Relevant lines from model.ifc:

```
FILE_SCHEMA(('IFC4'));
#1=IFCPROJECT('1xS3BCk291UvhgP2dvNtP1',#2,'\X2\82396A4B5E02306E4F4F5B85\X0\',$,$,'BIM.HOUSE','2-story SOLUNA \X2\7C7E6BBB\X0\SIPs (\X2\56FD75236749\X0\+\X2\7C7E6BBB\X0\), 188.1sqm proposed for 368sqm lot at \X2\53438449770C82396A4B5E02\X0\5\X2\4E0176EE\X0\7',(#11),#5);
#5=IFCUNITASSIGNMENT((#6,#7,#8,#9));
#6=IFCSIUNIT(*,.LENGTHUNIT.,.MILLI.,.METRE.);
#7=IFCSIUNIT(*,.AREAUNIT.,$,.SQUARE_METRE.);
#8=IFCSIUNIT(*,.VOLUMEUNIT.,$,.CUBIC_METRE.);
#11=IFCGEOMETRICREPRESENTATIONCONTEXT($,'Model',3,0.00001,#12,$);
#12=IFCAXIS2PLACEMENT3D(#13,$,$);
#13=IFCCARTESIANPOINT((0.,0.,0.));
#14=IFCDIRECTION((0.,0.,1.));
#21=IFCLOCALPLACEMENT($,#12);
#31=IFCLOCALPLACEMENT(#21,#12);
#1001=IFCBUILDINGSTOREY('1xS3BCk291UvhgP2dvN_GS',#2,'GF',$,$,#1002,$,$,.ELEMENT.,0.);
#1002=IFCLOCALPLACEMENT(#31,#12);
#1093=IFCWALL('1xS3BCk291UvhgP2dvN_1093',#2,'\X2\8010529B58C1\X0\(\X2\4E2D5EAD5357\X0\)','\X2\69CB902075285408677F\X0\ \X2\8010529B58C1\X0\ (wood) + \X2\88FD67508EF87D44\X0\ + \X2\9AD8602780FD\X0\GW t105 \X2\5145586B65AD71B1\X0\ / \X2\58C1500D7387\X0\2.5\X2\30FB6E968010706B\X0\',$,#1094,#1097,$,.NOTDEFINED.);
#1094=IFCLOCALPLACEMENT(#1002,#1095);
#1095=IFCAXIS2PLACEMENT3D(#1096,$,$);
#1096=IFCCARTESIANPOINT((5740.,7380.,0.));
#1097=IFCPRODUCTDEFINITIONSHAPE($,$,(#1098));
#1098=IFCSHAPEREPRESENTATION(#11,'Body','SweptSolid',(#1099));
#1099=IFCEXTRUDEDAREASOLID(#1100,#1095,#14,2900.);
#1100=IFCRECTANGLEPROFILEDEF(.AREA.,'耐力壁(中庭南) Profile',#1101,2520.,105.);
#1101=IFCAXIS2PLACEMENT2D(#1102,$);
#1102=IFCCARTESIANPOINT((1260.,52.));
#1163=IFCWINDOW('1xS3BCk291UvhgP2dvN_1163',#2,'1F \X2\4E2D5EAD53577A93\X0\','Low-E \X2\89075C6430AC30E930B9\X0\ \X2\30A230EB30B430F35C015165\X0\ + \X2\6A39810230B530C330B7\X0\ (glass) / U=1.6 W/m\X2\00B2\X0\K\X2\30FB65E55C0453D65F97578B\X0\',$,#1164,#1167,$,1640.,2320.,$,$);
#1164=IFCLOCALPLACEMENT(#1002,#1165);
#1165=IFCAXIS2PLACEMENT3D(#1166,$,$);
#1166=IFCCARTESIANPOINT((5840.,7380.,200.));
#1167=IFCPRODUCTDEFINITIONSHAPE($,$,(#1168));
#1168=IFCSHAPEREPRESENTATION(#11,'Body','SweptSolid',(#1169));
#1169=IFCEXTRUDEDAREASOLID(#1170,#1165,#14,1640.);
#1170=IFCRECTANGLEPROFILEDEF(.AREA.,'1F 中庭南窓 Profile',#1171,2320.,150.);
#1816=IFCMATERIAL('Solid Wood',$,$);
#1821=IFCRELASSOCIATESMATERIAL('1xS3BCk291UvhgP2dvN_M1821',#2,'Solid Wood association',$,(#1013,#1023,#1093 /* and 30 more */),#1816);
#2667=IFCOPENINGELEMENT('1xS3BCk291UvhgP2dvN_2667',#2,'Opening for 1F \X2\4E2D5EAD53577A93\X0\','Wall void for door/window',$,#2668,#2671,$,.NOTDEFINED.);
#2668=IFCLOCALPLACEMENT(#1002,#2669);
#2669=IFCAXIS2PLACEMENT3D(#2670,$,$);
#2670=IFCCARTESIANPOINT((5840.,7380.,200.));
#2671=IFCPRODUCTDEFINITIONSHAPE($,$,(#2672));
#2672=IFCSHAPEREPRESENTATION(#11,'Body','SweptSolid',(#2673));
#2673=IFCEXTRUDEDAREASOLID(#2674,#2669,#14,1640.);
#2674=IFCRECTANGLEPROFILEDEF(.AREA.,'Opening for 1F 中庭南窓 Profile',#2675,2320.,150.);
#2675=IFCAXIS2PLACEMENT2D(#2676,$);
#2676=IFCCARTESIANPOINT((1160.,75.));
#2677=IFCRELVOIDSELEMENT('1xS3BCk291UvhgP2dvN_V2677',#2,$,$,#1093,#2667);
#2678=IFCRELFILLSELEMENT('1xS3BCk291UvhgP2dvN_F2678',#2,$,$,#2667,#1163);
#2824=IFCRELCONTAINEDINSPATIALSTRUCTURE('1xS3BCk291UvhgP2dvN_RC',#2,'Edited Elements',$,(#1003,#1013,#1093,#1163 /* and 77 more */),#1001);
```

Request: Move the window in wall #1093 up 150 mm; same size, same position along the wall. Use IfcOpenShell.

```python
import numpy as np
import ifcopenshell
import ifcopenshell.api.geometry
import ifcopenshell.util.placement
import ifcopenshell.util.unit

model = ifcopenshell.open("model.ifc")
unit_scale = ifcopenshell.util.unit.calculate_unit_scale(model)

window = model.by_guid("1xS3BCk291UvhgP2dvN_1163")
opening = window.FillsVoids[0].RelatingOpeningElement
dz = 150.0

shift = np.array([0.0, 0.0, dz])
# The window is not placed relative to its opening, so move both.
for product in (opening, window):
    matrix = ifcopenshell.util.placement.get_local_placement(product.ObjectPlacement)
    matrix[:3, 3] += shift
    ifcopenshell.api.geometry.edit_object_placement(model, product=product, matrix=matrix, is_si=False)

print(f"moved by {dz * unit_scale:+.3f} m")

model.write("model_edited.ifc")
```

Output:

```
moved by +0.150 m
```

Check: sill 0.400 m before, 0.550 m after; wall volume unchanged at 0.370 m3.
